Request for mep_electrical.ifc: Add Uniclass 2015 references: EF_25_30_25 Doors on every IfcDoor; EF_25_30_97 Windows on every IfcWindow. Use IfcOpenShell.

First a look at what the model holds.

```python
import ifcopenshell

model = ifcopenshell.open("mep_electrical.ifc")
print(model.schema)
print("classifications:", [c.Name for c in model.by_type("IfcClassification")])
for ifc_class in ("IfcDoor", "IfcRoof", "IfcStair", "IfcWall", "IfcWindow"):
    print(ifc_class, len(model.by_type(ifc_class)))
```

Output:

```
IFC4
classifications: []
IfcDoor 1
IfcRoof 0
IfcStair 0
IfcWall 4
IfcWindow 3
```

```python
import ifcopenshell
import ifcopenshell.api.classification

model = ifcopenshell.open("mep_electrical.ifc")

system = ifcopenshell.api.classification.add_classification(model, classification="Uniclass 2015")

codes = {
    "IfcDoor": ("EF_25_30_25", "Doors"),
    "IfcWindow": ("EF_25_30_97", "Windows"),
}
for ifc_class, (code, name) in codes.items():
    products = model.by_type(ifc_class)
    ifcopenshell.api.classification.add_reference(
        model, products=products, classification=system, identification=code, name=name
    )
    print(code, len(products))

model.write("mep_electrical_rev.ifc")
```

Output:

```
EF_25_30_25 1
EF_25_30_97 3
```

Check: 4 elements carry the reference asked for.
